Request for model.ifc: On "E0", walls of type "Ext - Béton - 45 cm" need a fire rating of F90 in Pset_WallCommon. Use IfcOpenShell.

First a look at what the model holds.

```python
import ifcopenshell
import ifcopenshell.util.element

model = ifcopenshell.open("model.ifc")
print(model.schema)
storey = next(s for s in model.by_type("IfcBuildingStorey") if s.Name == "E0")
walls = [e for e in ifcopenshell.util.element.get_decomposition(storey) if e.is_a("IfcWall")]
seen = {}
for e in walls:
    element_type = ifcopenshell.util.element.get_type(e)
    key = (element_type.Name if element_type != e and element_type else None, ifcopenshell.util.element.get_pset(e, "Pset_WallCommon", "FireRating"))
    seen[key] = seen.get(key, 0) + 1
for (name, value), count in sorted(seen.items(), key=str):
    print(count, "x", name, "|", value)
```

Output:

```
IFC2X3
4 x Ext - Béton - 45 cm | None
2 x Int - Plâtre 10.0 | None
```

```python
import ifcopenshell
import ifcopenshell.api.pset
import ifcopenshell.util.element

model = ifcopenshell.open("model.ifc")

storey = next(s for s in model.by_type("IfcBuildingStorey") if s.Name == "E0")
walls = [e for e in ifcopenshell.util.element.get_decomposition(storey) if e.is_a("IfcWall")]

count = 0
for e in walls:
    element_type = ifcopenshell.util.element.get_type(e)
    if element_type in (None, e) or element_type.Name != "Ext - Béton - 45 cm":
        continue
    # add_pset returns the element's existing set when there is one.
    pset = ifcopenshell.api.pset.add_pset(model, product=e, name="Pset_WallCommon")
    ifcopenshell.api.pset.edit_pset(model, pset=pset, properties={"FireRating": "F90"})
    count += 1

print(count, "walls updated")

model.write("model_v2.ifc")
```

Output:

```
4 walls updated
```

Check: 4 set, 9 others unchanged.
